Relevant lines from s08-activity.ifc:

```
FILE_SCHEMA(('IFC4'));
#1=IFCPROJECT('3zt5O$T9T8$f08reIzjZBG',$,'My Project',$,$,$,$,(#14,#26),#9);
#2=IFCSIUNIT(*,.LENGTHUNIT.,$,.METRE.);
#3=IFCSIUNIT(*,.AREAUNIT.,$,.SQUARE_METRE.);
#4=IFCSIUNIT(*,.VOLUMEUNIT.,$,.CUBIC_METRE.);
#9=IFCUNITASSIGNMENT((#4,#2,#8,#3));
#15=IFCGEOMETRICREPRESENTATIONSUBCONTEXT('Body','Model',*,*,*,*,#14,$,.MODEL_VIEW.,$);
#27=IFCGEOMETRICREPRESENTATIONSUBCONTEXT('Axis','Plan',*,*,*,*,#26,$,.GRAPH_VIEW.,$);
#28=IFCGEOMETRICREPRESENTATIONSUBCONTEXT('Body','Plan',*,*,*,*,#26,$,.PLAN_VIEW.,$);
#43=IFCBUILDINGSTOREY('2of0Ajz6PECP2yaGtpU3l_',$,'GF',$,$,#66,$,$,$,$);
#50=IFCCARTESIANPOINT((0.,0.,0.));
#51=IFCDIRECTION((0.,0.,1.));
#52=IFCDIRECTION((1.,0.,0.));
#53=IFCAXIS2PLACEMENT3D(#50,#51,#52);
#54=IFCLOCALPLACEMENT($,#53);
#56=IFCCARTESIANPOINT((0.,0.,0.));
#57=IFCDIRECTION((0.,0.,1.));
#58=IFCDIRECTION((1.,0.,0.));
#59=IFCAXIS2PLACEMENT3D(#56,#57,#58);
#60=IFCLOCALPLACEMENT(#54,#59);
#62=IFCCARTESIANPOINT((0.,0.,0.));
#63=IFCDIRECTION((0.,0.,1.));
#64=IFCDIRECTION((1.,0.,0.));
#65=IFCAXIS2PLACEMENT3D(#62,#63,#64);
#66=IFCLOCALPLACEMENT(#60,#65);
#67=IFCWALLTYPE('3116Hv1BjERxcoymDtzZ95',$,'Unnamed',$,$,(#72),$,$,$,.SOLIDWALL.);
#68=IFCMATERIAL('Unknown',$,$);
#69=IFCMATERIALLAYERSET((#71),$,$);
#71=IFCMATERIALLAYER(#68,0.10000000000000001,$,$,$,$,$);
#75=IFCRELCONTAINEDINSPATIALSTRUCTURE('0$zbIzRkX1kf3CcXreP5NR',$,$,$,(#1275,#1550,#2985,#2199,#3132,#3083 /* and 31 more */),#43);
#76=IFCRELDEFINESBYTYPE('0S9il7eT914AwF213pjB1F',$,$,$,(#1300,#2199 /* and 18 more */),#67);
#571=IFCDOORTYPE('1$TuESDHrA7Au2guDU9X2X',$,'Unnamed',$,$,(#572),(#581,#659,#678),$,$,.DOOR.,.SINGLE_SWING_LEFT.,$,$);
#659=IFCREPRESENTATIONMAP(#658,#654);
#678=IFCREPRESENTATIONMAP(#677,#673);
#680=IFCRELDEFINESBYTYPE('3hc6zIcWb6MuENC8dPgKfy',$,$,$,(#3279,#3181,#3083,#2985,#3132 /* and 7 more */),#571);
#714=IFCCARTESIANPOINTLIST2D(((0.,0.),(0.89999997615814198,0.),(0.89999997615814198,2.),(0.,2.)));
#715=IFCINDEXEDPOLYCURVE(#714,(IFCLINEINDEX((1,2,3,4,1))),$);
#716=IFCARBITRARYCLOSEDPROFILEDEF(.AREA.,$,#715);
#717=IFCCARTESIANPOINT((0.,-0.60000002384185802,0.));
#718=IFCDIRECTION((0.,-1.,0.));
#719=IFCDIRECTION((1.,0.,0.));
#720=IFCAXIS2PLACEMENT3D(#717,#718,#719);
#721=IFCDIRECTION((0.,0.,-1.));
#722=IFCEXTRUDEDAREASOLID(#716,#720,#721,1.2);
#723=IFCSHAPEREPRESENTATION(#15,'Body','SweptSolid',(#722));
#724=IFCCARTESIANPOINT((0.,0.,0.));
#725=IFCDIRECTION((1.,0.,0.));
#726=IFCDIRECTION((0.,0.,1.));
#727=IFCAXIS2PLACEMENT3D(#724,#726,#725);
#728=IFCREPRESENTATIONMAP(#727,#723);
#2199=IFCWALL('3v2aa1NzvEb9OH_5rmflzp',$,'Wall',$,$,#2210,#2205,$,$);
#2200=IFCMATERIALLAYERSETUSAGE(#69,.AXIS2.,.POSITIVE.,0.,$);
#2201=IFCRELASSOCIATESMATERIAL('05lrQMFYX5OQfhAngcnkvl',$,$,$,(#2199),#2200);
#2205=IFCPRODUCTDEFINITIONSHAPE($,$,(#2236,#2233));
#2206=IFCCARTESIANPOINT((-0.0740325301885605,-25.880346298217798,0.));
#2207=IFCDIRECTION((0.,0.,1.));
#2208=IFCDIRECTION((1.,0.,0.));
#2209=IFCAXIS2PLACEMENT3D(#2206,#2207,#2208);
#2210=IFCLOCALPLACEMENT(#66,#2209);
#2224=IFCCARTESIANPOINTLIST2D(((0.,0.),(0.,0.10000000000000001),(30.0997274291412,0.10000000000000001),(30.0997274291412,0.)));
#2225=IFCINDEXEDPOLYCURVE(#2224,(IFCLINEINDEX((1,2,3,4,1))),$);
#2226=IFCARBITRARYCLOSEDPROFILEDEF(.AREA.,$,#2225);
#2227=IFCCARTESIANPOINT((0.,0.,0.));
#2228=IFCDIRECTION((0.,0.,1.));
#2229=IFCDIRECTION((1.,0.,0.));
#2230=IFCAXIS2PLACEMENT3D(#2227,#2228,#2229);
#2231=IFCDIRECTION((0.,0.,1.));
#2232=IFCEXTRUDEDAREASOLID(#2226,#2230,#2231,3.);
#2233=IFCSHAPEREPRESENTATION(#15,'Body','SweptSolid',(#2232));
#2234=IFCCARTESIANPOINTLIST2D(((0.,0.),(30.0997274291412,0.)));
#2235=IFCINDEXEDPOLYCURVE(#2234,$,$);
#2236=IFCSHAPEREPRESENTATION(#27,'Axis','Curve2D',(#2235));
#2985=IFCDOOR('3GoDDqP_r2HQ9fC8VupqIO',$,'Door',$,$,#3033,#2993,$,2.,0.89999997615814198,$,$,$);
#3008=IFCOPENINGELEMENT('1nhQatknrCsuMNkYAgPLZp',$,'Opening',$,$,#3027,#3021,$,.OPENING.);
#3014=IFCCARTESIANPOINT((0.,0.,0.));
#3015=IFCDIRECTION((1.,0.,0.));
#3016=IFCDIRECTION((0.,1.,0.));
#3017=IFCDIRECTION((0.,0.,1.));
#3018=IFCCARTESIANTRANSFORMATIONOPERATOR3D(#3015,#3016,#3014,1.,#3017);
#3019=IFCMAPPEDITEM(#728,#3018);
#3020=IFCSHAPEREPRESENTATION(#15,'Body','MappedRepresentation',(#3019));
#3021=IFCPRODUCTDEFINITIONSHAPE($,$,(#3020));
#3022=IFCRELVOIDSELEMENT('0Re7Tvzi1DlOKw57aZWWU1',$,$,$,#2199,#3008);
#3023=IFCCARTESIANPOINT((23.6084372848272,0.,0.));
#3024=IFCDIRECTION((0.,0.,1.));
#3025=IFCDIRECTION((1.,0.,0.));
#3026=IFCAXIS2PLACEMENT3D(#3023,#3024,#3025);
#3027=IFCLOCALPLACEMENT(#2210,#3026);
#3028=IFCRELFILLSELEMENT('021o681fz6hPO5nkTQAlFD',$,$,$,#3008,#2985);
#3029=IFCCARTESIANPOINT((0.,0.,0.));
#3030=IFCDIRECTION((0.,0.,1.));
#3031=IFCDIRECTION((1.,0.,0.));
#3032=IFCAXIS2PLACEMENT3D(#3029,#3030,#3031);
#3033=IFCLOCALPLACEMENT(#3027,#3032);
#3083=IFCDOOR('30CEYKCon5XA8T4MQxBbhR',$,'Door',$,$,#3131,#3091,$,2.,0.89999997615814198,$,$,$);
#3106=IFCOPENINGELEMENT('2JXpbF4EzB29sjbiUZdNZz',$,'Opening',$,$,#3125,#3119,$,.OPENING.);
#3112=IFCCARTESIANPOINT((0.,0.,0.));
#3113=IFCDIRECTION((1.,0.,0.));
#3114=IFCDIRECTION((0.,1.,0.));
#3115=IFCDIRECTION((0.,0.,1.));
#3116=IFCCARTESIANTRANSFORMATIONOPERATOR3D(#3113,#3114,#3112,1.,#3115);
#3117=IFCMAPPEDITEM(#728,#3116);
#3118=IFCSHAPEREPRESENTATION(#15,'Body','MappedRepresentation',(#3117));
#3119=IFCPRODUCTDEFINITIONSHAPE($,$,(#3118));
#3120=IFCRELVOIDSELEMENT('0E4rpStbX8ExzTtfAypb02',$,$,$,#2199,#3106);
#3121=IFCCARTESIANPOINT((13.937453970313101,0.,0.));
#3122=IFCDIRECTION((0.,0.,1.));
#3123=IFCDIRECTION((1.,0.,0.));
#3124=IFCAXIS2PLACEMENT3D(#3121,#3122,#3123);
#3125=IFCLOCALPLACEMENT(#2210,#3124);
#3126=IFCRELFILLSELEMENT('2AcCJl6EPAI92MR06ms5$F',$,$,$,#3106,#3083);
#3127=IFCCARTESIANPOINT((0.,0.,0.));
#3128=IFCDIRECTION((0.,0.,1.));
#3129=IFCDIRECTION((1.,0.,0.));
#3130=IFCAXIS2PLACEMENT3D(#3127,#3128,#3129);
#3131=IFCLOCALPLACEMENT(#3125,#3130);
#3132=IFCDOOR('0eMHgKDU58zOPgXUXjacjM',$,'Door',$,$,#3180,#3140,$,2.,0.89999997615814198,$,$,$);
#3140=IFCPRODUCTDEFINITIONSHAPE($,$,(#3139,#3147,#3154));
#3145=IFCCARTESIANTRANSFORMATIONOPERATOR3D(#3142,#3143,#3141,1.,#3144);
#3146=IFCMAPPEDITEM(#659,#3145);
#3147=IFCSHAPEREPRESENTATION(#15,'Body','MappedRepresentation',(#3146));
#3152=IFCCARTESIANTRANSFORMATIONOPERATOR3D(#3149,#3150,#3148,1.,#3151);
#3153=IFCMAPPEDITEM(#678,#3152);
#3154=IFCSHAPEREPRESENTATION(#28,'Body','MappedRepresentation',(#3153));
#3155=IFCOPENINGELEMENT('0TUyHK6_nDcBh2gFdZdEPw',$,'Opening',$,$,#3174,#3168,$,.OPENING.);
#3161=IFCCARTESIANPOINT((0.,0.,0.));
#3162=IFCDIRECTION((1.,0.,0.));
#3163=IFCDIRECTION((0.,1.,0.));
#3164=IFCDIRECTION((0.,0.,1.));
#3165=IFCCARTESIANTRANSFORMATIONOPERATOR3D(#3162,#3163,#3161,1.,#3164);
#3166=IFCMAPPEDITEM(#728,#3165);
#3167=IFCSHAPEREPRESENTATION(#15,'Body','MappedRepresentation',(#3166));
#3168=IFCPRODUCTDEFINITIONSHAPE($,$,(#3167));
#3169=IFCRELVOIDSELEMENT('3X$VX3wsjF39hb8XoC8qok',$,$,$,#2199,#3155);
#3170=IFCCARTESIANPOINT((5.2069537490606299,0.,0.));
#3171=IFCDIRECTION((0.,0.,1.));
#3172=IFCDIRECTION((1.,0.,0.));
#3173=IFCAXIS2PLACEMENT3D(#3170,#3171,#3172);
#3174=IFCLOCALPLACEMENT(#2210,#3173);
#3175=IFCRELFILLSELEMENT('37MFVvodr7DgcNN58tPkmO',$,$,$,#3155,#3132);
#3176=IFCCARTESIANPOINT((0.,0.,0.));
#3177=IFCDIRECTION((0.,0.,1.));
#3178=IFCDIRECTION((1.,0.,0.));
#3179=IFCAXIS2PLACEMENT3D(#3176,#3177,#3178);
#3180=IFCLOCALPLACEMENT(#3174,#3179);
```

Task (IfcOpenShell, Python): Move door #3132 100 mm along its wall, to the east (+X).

```python
import ifcopenshell
import ifcopenshell.api.geometry
import ifcopenshell.util.placement
import ifcopenshell.util.unit

model = ifcopenshell.open("s08-activity.ifc")
unit_scale = ifcopenshell.util.unit.calculate_unit_scale(model)

door = model.by_id(3132)
opening = door.FillsVoids[0].RelatingOpeningElement
wall = opening.VoidsElements[0].RelatingBuildingElement

wall_matrix = ifcopenshell.util.placement.get_local_placement(wall.ObjectPlacement)
shift = wall_matrix[:3, 0] * 0.1 / unit_scale
before = ifcopenshell.util.placement.get_local_placement(door.ObjectPlacement)[:3, 3].copy()

# The door is placed relative to its opening, so it follows when the opening moves.
matrix = ifcopenshell.util.placement.get_local_placement(opening.ObjectPlacement)
matrix[:3, 3] += shift
ifcopenshell.api.geometry.edit_object_placement(
    model, product=opening, matrix=matrix, is_si=False, should_transform_children=True
)

after = ifcopenshell.util.placement.get_local_placement(door.ObjectPlacement)[:3, 3]
print("door moved by", (after - before).round(3) + 0.0)

model.write("s08-activity_updated.ifc")
```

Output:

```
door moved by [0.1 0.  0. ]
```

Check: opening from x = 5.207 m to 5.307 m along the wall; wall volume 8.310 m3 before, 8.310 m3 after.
